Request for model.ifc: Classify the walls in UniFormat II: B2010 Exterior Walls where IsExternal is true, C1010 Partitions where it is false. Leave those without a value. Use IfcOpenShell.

First a look at what the model holds.

```python
import ifcopenshell
import ifcopenshell.util.element

model = ifcopenshell.open("model.ifc")
print(model.schema)
print("classifications:", [c.Name for c in model.by_type("IfcClassification")])
values = [ifcopenshell.util.element.get_pset(e, "Pset_WallCommon", "IsExternal") for e in model.by_type("IfcWall")]
for value in (True, False, None):
    print("IsExternal", value, values.count(value))
```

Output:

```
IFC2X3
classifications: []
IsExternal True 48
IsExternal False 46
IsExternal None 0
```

```python
import ifcopenshell
import ifcopenshell.api.classification
import ifcopenshell.util.element

model = ifcopenshell.open("model.ifc")

# IFC2X3 requires Source and Edition and has no link from the project to the system.
system = model.create_entity("IfcClassification", Source="ASTM", Edition="E1557", Name="UniFormat II")

walls = model.by_type("IfcWall")
external = {e: ifcopenshell.util.element.get_pset(e, "Pset_WallCommon", "IsExternal") for e in walls}
for flag, code, name in ((True, "B2010", "Exterior Walls"), (False, "C1010", "Partitions")):
    products = [e for e in walls if external[e] is flag]
    ifcopenshell.api.classification.add_reference(
        model, products=products, classification=system, identification=code, name=name
    )
    print(code, len(products))

model.write("model_rev.ifc")
```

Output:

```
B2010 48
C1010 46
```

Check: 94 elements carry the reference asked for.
